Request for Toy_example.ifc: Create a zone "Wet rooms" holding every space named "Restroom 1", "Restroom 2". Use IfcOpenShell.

First a look at what the model holds.

```python
import ifcopenshell

model = ifcopenshell.open("Toy_example.ifc")
print(model.schema)
seen = {}
for space in model.by_type("IfcSpace"):
    seen[space.LongName] = seen.get(space.LongName, 0) + 1
for name, count in sorted(seen.items(), key=str):
    print(count, "x", name)
print("zones:", [z.Name for z in model.by_type("IfcZone")][:20])
```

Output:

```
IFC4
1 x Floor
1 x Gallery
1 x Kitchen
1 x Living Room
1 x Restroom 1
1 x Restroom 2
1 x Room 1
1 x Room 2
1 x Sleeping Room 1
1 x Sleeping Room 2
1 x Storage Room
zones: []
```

```python
import ifcopenshell
import ifcopenshell.api.group
import ifcopenshell.api.root

model = ifcopenshell.open("Toy_example.ifc")

names = {"Restroom 1", "Restroom 2"}
spaces = [s for s in model.by_type("IfcSpace") if s.LongName in names]

zone = ifcopenshell.api.root.create_entity(model, ifc_class="IfcZone", name="Wet rooms")
ifcopenshell.api.group.assign_group(model, products=spaces, group=zone)
print(len(spaces), "spaces in", zone.Name)

model.write("Toy_example-out.ifc")
```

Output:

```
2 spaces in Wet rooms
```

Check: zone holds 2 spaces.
